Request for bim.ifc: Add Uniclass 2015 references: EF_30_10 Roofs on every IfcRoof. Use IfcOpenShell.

First a look at what the model holds.

```python
import ifcopenshell

model = ifcopenshell.open("bim.ifc")
print(model.schema)
print("classifications:", [c.Name for c in model.by_type("IfcClassification")])
for ifc_class in ("IfcDoor", "IfcRoof", "IfcStair", "IfcWall", "IfcWindow"):
    print(ifc_class, len(model.by_type(ifc_class)))
```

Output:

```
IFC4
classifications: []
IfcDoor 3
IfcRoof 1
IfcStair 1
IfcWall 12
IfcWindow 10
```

```python
import ifcopenshell
import ifcopenshell.api.classification

model = ifcopenshell.open("bim.ifc")

system = ifcopenshell.api.classification.add_classification(model, classification="Uniclass 2015")

codes = {
    "IfcRoof": ("EF_30_10", "Roofs"),
}
for ifc_class, (code, name) in codes.items():
    products = model.by_type(ifc_class)
    ifcopenshell.api.classification.add_reference(
        model, products=products, classification=system, identification=code, name=name
    )
    print(code, len(products))

model.write("bim_v2.ifc")
```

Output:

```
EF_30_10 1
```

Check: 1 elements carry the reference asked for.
